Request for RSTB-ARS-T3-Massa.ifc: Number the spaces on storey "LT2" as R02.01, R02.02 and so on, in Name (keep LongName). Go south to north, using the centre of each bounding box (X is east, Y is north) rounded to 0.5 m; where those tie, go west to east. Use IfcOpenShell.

First a look at what the model holds.

```python
import ifcopenshell
import ifcopenshell.util.element
import ifcopenshell.util.placement

model = ifcopenshell.open("RSTB-ARS-T3-Massa.ifc")
print(model.schema)
storey = next(s for s in model.by_type("IfcBuildingStorey") if s.Name == "LT2")
spaces = [e for e in ifcopenshell.util.element.get_decomposition(storey) if e.is_a("IfcSpace")]
for e in sorted(spaces, key=lambda e: e.id()):
    origin = ifcopenshell.util.placement.get_local_placement(e.ObjectPlacement)[:3, 3]
    print(e.id(), e.Name, e.LongName, origin.round(2) + 0.0, sep=" | ")
```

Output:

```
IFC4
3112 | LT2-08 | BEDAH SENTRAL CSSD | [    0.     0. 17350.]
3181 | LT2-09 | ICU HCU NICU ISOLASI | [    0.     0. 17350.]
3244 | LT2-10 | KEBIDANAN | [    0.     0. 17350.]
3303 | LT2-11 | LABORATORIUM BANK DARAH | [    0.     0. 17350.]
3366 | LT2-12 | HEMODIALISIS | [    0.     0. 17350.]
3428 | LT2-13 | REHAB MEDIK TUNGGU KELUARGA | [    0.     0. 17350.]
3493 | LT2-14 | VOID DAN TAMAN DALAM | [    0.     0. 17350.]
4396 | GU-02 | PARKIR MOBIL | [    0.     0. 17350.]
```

```python
import ifcopenshell
import ifcopenshell.geom
import ifcopenshell.util.element
import ifcopenshell.util.shape

model = ifcopenshell.open("RSTB-ARS-T3-Massa.ifc")
settings = ifcopenshell.geom.settings()
settings.set("use-world-coords", True)


def centre(element):
    shape = ifcopenshell.geom.create_shape(settings, element)
    return ifcopenshell.util.shape.get_bbox_centroid(shape.geometry)


storey = next(s for s in model.by_type("IfcBuildingStorey") if s.Name == "LT2")
spaces = [e for e in ifcopenshell.util.element.get_decomposition(storey) if e.is_a("IfcSpace")]

# Insertion points can sit at a corner or the storey origin, so sort by the geometry (in metres).
centres = {e: centre(e) for e in spaces}
spaces.sort(key=lambda e: (round(centres[e][1] / 0.5), centres[e][0]))

for i, e in enumerate(spaces, start=1):
    number = f"R02.{i:02d}"
    e.Name = number
    print(e.id(), number)

model.write("RSTB-ARS-T3-Massa_v2.ifc")
```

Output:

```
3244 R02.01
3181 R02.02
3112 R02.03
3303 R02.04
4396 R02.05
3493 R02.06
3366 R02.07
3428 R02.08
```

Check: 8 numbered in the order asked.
